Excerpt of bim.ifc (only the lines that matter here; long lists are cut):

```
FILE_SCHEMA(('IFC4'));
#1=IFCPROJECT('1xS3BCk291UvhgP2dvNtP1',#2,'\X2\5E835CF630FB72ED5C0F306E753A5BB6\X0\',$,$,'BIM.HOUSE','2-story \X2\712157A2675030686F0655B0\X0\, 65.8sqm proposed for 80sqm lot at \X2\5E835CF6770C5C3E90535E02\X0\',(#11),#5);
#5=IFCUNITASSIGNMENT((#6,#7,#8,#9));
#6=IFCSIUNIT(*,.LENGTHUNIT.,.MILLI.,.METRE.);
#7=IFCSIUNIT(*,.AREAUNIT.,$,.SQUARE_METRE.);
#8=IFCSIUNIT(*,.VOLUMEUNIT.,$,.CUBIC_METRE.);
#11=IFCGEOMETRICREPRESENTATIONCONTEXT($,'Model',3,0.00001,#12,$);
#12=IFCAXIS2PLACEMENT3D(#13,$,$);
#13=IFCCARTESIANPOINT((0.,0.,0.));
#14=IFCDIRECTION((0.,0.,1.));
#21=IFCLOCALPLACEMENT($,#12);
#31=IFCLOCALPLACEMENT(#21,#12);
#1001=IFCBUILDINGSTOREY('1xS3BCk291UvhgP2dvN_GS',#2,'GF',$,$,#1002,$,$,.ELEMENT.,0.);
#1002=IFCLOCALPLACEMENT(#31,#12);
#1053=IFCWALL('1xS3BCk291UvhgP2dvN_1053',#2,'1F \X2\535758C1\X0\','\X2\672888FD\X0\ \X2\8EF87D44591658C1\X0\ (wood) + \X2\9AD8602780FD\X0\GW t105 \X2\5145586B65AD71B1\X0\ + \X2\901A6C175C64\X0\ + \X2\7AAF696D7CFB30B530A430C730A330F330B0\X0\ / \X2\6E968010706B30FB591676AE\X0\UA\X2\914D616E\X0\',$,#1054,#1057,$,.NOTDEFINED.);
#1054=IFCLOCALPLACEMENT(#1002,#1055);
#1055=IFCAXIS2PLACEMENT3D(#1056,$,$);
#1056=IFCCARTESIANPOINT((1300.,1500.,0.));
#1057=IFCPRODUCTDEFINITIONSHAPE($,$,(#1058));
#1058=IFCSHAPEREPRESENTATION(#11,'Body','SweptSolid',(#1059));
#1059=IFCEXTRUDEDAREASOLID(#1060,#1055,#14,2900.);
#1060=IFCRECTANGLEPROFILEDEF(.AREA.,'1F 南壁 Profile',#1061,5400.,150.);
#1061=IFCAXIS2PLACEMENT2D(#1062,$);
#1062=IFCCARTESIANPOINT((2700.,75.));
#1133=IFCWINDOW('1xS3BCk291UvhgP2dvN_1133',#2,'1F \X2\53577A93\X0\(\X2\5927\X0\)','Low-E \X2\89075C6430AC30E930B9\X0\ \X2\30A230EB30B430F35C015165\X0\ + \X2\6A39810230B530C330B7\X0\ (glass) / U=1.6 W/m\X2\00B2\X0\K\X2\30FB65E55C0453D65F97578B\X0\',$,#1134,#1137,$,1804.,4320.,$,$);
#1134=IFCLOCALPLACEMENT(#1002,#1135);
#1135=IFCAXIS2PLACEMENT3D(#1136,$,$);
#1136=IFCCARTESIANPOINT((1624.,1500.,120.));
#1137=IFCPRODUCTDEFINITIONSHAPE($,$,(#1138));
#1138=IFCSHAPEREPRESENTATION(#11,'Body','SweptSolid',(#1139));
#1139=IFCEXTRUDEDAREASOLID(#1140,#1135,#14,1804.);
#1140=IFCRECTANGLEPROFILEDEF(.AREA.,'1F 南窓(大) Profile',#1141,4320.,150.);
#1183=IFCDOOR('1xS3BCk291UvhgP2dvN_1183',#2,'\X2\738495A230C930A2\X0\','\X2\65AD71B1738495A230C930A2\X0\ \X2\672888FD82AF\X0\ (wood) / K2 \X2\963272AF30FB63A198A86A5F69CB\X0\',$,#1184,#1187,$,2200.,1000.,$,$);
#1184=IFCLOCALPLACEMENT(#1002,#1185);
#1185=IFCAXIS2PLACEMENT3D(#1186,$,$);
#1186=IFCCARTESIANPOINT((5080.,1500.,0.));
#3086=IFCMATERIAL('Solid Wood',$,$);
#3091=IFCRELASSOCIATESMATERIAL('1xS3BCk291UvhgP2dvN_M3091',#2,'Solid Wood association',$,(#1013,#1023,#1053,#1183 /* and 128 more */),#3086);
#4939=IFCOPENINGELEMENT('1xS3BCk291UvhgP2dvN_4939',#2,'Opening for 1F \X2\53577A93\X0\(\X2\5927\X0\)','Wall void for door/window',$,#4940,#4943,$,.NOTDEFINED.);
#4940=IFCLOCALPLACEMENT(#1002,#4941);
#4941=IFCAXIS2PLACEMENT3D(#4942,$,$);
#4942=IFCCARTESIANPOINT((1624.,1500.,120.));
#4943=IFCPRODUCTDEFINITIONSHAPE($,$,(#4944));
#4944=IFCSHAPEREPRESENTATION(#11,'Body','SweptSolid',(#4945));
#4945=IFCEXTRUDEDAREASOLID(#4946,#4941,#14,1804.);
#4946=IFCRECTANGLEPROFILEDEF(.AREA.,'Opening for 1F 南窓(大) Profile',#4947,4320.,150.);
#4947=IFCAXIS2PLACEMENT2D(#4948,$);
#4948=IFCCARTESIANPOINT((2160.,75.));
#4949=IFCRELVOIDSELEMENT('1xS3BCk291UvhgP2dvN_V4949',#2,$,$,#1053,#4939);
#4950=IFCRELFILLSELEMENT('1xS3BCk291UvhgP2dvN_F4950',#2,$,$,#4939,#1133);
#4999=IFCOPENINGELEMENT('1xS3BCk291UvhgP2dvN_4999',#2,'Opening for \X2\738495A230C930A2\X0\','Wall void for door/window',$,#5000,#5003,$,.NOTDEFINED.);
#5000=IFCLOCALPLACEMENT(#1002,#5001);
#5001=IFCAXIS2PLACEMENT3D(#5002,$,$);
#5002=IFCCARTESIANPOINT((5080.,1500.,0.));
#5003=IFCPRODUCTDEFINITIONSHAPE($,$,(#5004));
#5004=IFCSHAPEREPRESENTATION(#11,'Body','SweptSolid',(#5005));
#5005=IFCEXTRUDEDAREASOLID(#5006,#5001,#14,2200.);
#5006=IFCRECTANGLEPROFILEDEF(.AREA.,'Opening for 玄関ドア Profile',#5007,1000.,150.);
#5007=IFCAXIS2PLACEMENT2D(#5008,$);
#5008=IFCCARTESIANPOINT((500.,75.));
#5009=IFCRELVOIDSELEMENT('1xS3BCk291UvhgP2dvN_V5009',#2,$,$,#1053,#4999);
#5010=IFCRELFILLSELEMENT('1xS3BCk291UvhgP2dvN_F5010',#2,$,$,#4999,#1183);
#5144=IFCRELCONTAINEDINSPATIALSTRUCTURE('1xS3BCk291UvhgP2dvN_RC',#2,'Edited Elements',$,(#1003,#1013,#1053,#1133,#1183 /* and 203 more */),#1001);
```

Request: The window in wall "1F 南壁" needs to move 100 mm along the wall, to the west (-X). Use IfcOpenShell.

```python
import ifcopenshell
import ifcopenshell.api.geometry
import ifcopenshell.util.placement
import ifcopenshell.util.unit

model = ifcopenshell.open("bim.ifc")
unit_scale = ifcopenshell.util.unit.calculate_unit_scale(model)

window = model.by_guid("1xS3BCk291UvhgP2dvN_1133")
opening = window.FillsVoids[0].RelatingOpeningElement
wall = opening.VoidsElements[0].RelatingBuildingElement

wall_matrix = ifcopenshell.util.placement.get_local_placement(wall.ObjectPlacement)
shift = wall_matrix[:3, 0] * -0.1 / unit_scale
before = ifcopenshell.util.placement.get_local_placement(window.ObjectPlacement)[:3, 3].copy()

# The window is not placed relative to its opening, so move both.
for product in (opening, window):
    matrix = ifcopenshell.util.placement.get_local_placement(product.ObjectPlacement)
    matrix[:3, 3] += shift
    ifcopenshell.api.geometry.edit_object_placement(model, product=product, matrix=matrix, is_si=False)

after = ifcopenshell.util.placement.get_local_placement(window.ObjectPlacement)[:3, 3]
print("window moved by", (after - before).round(3) + 0.0)

model.write("bim_edited.ifc")
```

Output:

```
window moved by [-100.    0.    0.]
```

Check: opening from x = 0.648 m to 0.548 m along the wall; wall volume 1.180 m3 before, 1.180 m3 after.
